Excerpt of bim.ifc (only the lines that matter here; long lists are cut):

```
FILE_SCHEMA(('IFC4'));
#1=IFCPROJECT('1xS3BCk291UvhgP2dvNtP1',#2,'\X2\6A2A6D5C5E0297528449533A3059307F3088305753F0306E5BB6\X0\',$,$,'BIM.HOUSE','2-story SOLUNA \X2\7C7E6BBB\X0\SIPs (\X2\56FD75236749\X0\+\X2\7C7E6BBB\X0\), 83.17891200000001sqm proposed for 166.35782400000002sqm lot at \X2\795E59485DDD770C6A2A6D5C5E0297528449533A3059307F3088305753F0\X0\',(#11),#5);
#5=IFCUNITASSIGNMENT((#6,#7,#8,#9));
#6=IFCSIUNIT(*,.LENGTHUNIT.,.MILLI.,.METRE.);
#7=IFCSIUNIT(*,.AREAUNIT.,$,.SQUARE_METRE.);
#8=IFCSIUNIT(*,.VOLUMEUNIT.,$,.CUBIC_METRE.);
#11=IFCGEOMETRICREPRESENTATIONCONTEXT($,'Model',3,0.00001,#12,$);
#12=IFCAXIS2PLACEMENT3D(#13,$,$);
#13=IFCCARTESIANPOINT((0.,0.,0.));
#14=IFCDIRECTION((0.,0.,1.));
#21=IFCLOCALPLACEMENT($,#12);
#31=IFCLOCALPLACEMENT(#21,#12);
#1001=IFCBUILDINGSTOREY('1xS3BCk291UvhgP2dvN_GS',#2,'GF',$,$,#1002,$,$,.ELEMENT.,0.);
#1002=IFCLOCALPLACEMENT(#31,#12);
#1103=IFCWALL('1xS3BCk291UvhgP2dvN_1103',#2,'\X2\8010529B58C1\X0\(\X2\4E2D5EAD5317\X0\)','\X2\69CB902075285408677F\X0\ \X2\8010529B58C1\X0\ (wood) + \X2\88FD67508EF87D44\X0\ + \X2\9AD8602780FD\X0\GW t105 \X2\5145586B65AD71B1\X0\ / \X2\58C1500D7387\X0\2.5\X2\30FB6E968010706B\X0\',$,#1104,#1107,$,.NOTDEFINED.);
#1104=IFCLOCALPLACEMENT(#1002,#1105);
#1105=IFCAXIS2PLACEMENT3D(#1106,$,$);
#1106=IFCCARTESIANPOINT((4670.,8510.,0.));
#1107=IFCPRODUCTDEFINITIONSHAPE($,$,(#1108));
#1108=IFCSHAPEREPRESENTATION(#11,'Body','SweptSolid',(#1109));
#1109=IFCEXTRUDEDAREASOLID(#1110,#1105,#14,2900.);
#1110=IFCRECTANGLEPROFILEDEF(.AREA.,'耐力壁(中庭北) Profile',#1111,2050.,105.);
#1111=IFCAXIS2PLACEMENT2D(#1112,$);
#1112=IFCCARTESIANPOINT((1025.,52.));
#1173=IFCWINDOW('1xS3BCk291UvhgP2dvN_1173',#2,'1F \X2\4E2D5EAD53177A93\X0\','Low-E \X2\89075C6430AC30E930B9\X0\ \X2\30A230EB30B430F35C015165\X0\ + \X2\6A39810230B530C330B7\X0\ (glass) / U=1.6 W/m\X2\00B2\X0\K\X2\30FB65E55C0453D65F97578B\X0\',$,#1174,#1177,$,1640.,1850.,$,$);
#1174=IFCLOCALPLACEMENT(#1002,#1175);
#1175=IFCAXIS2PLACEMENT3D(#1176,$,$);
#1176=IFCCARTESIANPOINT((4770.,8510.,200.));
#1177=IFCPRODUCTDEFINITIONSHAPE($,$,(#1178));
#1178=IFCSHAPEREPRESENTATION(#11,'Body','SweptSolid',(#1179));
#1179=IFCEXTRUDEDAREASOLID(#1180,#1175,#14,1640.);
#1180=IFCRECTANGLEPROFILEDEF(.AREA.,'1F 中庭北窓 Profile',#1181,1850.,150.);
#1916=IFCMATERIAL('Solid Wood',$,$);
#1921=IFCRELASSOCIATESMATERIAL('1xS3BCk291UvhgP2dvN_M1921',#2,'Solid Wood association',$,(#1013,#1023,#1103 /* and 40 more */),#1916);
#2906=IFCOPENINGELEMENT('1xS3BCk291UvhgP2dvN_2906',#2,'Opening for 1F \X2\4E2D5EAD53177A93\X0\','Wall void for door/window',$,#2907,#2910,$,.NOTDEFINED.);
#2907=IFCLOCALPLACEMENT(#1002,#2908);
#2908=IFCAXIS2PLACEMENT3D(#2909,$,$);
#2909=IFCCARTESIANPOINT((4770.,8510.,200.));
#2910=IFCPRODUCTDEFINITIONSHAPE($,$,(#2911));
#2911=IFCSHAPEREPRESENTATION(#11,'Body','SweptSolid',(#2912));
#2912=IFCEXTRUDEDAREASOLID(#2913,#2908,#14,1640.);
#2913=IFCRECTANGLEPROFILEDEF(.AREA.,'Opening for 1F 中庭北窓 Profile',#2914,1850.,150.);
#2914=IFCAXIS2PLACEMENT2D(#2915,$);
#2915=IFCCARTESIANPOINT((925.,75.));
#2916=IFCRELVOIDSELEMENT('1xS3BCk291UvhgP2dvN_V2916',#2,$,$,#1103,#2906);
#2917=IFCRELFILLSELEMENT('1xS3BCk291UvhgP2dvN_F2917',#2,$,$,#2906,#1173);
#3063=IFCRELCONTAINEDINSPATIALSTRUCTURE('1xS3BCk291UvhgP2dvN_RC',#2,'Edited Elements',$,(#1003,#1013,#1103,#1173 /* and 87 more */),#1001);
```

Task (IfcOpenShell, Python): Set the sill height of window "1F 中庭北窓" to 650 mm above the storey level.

```python
import numpy as np
import ifcopenshell
import ifcopenshell.api.geometry
import ifcopenshell.geom
import ifcopenshell.util.element
import ifcopenshell.util.placement
import ifcopenshell.util.shape
import ifcopenshell.util.unit

model = ifcopenshell.open("bim.ifc")
unit_scale = ifcopenshell.util.unit.calculate_unit_scale(model)

window = model.by_guid("1xS3BCk291UvhgP2dvN_1173")
opening = window.FillsVoids[0].RelatingOpeningElement
storey = ifcopenshell.util.element.get_container(window, ifc_class="IfcBuildingStorey")
level = ifcopenshell.util.placement.get_local_placement(storey.ObjectPlacement)[2, 3]

# The opening's origin need not be at the sill, so measure its lowest point.
shape = ifcopenshell.geom.create_shape(ifcopenshell.geom.settings(), opening)
bottom = ifcopenshell.util.shape.get_shape_bottom_elevation(shape, shape.geometry) / unit_scale
dz = level + 0.65 / unit_scale - bottom

shift = np.array([0.0, 0.0, dz])
# The window is not placed relative to its opening, so move both.
for product in (opening, window):
    matrix = ifcopenshell.util.placement.get_local_placement(product.ObjectPlacement)
    matrix[:3, 3] += shift
    ifcopenshell.api.geometry.edit_object_placement(model, product=product, matrix=matrix, is_si=False)

print(f"moved by {dz * unit_scale:+.3f} m")

model.write("bim_rev.ifc")
```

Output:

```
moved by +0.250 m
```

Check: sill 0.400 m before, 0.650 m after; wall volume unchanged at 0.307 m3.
